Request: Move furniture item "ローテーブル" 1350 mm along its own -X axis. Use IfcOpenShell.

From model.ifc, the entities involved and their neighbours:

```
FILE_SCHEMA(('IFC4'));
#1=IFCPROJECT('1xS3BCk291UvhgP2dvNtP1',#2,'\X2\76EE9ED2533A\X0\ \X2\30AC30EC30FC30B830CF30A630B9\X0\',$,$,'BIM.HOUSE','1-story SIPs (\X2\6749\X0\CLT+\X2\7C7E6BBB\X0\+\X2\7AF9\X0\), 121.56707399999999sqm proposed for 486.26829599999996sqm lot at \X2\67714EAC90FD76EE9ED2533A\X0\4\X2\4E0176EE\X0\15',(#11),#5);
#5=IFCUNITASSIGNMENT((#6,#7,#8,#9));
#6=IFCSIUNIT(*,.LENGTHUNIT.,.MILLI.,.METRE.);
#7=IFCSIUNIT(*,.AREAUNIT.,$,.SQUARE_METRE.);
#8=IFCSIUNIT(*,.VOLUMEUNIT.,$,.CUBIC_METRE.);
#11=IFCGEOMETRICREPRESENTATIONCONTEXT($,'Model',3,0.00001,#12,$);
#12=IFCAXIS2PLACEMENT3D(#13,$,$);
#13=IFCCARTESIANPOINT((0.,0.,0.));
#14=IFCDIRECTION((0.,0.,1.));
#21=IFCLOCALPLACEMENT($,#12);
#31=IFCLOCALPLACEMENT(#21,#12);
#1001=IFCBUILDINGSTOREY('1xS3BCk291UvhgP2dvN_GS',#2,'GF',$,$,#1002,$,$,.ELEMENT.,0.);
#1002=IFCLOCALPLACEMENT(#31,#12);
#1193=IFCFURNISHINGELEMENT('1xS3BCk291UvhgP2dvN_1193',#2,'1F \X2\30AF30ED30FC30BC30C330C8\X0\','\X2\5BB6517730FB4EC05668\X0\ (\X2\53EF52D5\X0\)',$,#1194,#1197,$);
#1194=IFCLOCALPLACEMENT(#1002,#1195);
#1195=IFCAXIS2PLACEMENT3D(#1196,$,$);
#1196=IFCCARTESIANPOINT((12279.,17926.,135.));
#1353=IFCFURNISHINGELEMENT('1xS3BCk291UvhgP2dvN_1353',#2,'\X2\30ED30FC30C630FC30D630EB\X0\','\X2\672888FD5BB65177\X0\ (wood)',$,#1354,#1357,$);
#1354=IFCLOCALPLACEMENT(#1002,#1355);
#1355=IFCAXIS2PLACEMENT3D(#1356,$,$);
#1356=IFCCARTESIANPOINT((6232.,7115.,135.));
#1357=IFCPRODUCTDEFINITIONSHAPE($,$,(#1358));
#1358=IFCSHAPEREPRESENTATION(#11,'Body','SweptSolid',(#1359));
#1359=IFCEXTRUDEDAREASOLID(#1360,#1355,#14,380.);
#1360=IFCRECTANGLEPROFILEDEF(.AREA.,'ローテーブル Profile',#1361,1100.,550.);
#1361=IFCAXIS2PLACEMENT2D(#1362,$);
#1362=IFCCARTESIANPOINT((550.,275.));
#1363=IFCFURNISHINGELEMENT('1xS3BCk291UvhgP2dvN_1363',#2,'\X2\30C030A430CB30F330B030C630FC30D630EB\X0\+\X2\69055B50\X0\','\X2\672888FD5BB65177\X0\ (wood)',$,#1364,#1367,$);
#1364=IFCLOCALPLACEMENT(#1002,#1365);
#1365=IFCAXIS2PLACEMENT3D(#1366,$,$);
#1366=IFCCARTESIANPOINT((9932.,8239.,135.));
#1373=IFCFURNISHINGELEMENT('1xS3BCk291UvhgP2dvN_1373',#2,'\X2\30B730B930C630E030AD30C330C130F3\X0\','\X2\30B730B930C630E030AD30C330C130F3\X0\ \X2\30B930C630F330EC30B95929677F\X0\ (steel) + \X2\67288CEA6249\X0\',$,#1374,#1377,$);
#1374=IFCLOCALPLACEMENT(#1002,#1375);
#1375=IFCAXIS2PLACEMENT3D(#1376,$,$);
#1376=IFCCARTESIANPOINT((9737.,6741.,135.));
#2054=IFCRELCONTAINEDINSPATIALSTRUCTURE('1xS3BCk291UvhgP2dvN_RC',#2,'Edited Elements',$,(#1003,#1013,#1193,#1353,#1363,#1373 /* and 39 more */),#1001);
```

```python
import ifcopenshell
import ifcopenshell.api.geometry
import ifcopenshell.util.placement
import ifcopenshell.util.unit

model = ifcopenshell.open("model.ifc")
unit_scale = ifcopenshell.util.unit.calculate_unit_scale(model)

item = model.by_guid("1xS3BCk291UvhgP2dvN_1353")
matrix = ifcopenshell.util.placement.get_local_placement(item.ObjectPlacement)
matrix[:3, 3] -= matrix[:3, 0] * 1.35 / unit_scale
ifcopenshell.api.geometry.edit_object_placement(model, product=item, matrix=matrix, is_si=False)

print(ifcopenshell.util.placement.get_local_placement(item.ObjectPlacement).round(3) + 0.0)

model.write("model_updated.ifc")
```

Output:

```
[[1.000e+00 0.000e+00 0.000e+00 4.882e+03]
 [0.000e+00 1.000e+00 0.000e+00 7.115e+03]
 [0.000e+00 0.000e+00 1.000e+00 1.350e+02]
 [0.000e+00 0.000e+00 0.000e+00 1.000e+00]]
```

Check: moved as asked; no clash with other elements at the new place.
